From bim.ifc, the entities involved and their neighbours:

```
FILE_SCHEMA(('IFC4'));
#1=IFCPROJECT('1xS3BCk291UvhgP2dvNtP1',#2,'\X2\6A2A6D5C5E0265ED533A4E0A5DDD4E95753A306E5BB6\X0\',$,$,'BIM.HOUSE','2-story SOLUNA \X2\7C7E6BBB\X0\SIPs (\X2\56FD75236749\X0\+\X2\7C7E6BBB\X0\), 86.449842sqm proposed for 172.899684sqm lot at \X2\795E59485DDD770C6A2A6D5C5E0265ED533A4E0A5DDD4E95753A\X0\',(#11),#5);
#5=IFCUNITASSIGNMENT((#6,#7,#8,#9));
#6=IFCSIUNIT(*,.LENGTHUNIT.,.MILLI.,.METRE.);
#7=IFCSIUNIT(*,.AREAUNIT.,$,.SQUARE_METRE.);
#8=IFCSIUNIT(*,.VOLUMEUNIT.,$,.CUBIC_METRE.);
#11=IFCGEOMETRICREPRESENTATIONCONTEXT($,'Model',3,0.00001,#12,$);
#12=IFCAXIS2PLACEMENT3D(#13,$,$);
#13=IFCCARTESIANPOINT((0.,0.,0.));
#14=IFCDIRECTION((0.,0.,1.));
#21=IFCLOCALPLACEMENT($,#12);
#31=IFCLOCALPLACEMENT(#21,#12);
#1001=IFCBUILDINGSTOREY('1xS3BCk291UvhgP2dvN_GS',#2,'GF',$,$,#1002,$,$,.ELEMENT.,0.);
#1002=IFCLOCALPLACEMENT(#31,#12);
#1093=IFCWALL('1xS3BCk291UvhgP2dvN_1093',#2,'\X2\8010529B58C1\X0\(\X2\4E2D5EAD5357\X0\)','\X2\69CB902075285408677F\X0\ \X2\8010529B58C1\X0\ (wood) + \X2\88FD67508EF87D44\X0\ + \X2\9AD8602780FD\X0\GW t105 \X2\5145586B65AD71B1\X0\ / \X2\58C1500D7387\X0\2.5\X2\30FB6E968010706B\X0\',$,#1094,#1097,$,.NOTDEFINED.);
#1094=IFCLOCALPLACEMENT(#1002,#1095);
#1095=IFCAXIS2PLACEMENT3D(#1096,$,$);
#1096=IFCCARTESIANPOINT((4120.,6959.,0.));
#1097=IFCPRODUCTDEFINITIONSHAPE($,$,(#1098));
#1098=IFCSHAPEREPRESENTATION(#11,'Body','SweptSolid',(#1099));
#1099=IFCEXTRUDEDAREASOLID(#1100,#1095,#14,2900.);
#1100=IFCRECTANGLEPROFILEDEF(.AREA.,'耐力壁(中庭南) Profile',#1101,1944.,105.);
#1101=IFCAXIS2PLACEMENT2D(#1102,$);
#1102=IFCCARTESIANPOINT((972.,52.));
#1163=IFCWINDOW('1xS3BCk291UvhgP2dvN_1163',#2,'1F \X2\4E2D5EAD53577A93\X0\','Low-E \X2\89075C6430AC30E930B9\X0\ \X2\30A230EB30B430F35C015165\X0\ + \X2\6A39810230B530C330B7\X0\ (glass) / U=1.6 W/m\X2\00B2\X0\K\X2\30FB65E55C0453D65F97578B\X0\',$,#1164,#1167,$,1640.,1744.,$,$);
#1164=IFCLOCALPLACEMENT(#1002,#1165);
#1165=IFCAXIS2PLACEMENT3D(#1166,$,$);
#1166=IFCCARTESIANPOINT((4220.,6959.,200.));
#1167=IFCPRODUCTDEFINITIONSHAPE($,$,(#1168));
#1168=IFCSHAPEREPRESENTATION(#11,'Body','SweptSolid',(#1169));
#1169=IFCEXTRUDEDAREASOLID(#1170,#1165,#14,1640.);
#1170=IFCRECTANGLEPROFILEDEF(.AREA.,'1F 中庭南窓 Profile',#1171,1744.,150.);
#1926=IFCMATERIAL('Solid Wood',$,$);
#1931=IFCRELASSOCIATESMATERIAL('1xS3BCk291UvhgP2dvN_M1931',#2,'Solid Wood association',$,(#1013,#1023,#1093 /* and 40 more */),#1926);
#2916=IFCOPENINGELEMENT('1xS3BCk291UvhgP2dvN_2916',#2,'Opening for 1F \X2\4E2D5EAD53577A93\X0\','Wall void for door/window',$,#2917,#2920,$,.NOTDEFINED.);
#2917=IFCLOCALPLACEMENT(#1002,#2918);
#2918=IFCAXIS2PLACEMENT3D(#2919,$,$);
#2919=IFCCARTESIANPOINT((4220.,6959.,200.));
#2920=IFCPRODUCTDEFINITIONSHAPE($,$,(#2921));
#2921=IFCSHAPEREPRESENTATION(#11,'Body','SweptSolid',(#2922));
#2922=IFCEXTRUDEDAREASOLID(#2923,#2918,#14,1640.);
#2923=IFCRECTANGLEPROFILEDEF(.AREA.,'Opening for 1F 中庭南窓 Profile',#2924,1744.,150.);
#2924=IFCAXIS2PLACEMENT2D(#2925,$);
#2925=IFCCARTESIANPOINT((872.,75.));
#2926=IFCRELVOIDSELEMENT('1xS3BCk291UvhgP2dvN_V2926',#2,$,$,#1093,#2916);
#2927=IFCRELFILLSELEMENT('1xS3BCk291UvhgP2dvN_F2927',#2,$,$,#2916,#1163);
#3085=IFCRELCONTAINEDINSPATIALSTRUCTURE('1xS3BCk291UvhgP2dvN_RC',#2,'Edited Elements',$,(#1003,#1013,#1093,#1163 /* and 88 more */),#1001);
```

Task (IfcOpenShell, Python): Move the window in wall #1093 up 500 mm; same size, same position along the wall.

```python
import numpy as np
import ifcopenshell
import ifcopenshell.api.geometry
import ifcopenshell.util.placement
import ifcopenshell.util.unit

model = ifcopenshell.open("bim.ifc")
unit_scale = ifcopenshell.util.unit.calculate_unit_scale(model)

window = model.by_id(1163)
opening = window.FillsVoids[0].RelatingOpeningElement
dz = 0.5 / unit_scale

shift = np.array([0.0, 0.0, dz])
# The window is not placed relative to its opening, so move both.
for product in (opening, window):
    matrix = ifcopenshell.util.placement.get_local_placement(product.ObjectPlacement)
    matrix[:3, 3] += shift
    ifcopenshell.api.geometry.edit_object_placement(model, product=product, matrix=matrix, is_si=False)

print(f"moved by {dz * unit_scale:+.3f} m")

model.write("bim_updated.ifc")
```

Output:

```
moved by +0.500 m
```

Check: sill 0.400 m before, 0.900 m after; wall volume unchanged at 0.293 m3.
